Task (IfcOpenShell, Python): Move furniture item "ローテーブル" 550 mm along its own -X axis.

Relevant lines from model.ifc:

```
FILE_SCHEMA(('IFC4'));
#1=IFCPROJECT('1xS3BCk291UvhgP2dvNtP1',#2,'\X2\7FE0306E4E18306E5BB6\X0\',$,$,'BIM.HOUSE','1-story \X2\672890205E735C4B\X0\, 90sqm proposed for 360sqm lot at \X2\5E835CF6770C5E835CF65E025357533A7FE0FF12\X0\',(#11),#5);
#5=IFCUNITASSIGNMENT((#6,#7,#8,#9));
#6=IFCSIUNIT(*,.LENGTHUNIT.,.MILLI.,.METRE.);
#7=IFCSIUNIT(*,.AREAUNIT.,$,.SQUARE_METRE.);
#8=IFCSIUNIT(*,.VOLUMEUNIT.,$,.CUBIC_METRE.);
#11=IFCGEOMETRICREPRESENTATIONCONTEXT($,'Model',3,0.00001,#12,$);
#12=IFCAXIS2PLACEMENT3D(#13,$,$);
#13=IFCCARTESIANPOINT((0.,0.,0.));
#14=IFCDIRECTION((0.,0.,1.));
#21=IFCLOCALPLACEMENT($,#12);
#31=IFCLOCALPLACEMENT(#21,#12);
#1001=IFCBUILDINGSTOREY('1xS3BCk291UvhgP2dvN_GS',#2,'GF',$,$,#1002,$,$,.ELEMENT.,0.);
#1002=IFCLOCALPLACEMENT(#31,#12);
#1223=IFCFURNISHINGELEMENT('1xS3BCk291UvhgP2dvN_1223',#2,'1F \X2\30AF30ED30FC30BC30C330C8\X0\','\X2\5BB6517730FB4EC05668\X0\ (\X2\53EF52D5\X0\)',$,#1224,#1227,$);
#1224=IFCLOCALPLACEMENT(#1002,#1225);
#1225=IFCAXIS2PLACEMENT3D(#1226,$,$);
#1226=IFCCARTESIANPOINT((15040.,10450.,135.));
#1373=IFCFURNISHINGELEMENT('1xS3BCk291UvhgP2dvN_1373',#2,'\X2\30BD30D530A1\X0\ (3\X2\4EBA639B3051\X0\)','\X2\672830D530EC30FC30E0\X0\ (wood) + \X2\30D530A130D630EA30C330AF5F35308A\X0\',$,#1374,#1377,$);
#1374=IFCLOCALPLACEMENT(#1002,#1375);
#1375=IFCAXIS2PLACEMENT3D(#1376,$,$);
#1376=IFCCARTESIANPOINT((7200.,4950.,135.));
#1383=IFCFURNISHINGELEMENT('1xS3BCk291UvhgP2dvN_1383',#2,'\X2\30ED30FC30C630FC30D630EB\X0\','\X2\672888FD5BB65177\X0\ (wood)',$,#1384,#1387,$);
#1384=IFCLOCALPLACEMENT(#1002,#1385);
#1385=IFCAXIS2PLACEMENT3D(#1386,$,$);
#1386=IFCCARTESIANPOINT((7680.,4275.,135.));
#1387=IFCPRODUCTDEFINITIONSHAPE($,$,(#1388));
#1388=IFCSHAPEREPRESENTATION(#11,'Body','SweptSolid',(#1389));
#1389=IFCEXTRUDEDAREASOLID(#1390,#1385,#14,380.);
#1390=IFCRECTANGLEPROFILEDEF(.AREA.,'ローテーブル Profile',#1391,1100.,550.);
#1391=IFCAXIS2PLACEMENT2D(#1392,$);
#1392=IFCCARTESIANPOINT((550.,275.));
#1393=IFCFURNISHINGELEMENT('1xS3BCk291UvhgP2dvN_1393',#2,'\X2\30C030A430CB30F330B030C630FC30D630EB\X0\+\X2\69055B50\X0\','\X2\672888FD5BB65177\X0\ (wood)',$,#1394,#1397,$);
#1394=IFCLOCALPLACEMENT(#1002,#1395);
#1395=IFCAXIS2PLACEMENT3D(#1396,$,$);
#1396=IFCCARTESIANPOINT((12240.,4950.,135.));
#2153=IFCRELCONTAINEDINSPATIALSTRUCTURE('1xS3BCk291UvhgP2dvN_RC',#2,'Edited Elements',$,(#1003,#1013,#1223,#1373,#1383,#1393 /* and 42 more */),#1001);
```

```python
import ifcopenshell
import ifcopenshell.api.geometry
import ifcopenshell.util.placement

model = ifcopenshell.open("model.ifc")

item = model.by_guid("1xS3BCk291UvhgP2dvN_1383")
matrix = ifcopenshell.util.placement.get_local_placement(item.ObjectPlacement)
matrix[:3, 3] -= matrix[:3, 0] * 550.0
ifcopenshell.api.geometry.edit_object_placement(model, product=item, matrix=matrix, is_si=False)

print(ifcopenshell.util.placement.get_local_placement(item.ObjectPlacement).round(3) + 0.0)

model.write("model_edited.ifc")
```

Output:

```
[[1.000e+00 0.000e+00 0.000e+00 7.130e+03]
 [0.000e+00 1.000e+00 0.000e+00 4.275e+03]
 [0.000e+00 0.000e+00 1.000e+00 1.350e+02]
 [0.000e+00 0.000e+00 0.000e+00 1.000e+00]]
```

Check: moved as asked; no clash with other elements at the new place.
